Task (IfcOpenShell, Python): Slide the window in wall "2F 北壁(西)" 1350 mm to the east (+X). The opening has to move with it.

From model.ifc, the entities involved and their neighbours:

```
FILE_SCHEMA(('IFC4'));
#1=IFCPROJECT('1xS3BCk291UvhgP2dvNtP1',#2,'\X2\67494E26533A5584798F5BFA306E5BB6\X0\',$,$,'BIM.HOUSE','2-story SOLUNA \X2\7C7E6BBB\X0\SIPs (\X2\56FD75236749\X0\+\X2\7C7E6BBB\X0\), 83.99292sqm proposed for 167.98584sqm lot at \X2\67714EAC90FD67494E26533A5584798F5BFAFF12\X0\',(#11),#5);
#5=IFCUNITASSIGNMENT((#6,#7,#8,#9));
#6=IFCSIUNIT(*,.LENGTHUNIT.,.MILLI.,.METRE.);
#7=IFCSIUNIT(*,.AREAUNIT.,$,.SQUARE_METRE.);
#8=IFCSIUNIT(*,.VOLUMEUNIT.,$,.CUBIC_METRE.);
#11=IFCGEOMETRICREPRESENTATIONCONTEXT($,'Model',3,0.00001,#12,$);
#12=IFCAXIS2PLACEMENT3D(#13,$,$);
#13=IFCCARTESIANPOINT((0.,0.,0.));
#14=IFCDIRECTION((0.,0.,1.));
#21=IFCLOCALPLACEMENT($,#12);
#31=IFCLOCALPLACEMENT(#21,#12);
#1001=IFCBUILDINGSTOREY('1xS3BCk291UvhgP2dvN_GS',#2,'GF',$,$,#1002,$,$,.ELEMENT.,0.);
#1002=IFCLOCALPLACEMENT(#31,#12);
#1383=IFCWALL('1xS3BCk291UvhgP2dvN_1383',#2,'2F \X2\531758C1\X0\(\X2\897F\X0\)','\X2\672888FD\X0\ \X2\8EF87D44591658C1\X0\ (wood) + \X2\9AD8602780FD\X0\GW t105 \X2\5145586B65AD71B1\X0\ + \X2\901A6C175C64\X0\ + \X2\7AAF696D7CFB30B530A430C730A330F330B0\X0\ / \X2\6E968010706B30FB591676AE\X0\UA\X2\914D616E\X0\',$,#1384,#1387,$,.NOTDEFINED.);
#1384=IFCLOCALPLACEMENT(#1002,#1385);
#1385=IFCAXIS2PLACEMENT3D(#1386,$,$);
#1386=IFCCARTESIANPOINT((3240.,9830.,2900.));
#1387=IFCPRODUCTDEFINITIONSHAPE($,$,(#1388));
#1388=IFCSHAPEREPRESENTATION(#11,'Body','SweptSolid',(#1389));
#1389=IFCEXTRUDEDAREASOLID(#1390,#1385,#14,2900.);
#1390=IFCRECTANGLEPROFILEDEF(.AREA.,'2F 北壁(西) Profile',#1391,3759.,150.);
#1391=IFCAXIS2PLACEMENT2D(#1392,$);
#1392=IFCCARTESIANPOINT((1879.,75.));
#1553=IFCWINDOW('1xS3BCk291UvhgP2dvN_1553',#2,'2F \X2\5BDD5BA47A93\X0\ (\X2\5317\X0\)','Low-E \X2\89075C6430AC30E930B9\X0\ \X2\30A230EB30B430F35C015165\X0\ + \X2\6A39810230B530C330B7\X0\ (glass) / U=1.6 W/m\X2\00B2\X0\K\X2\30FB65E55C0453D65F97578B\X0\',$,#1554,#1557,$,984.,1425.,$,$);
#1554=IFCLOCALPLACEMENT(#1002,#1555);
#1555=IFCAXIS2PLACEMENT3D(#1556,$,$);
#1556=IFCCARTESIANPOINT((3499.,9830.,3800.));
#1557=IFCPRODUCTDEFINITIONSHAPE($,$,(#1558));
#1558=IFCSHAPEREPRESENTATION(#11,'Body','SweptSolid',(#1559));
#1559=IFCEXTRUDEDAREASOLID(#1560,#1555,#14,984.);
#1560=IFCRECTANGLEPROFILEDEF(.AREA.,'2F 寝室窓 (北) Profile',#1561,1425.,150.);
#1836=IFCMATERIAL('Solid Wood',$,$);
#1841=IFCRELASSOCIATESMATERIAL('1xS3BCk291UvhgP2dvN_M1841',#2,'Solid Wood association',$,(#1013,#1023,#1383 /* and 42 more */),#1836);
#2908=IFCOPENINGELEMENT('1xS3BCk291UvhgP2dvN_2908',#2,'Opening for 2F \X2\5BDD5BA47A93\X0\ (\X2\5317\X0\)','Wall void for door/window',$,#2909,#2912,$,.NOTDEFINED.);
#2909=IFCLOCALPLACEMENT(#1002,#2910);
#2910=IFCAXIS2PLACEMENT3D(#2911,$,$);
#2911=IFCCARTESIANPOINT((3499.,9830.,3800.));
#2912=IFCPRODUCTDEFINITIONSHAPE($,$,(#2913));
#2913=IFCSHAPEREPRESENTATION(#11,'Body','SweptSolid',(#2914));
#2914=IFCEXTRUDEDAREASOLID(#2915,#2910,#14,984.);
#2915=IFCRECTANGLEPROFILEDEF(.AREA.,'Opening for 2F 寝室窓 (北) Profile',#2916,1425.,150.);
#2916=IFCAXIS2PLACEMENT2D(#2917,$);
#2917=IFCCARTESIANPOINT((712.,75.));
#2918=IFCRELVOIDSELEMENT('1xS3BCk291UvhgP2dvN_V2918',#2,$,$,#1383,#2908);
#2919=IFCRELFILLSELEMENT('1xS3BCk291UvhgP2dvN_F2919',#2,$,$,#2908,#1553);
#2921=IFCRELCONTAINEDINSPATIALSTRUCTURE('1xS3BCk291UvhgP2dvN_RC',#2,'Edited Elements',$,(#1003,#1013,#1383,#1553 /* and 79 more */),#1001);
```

```python
import ifcopenshell
import ifcopenshell.api.geometry
import ifcopenshell.util.placement

model = ifcopenshell.open("model.ifc")

window = model.by_guid("1xS3BCk291UvhgP2dvN_1553")
opening = window.FillsVoids[0].RelatingOpeningElement
wall = opening.VoidsElements[0].RelatingBuildingElement

wall_matrix = ifcopenshell.util.placement.get_local_placement(wall.ObjectPlacement)
shift = wall_matrix[:3, 0] * 1350.0
before = ifcopenshell.util.placement.get_local_placement(window.ObjectPlacement)[:3, 3].copy()

# The window is not placed relative to its opening, so move both.
for product in (opening, window):
    matrix = ifcopenshell.util.placement.get_local_placement(product.ObjectPlacement)
    matrix[:3, 3] += shift
    ifcopenshell.api.geometry.edit_object_placement(model, product=product, matrix=matrix, is_si=False)

after = ifcopenshell.util.placement.get_local_placement(window.ObjectPlacement)[:3, 3]
print("window moved by", (after - before).round(3) + 0.0)

model.write("model-out.ifc")
```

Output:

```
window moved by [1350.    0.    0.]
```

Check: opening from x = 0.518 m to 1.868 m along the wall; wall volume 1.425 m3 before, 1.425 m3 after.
